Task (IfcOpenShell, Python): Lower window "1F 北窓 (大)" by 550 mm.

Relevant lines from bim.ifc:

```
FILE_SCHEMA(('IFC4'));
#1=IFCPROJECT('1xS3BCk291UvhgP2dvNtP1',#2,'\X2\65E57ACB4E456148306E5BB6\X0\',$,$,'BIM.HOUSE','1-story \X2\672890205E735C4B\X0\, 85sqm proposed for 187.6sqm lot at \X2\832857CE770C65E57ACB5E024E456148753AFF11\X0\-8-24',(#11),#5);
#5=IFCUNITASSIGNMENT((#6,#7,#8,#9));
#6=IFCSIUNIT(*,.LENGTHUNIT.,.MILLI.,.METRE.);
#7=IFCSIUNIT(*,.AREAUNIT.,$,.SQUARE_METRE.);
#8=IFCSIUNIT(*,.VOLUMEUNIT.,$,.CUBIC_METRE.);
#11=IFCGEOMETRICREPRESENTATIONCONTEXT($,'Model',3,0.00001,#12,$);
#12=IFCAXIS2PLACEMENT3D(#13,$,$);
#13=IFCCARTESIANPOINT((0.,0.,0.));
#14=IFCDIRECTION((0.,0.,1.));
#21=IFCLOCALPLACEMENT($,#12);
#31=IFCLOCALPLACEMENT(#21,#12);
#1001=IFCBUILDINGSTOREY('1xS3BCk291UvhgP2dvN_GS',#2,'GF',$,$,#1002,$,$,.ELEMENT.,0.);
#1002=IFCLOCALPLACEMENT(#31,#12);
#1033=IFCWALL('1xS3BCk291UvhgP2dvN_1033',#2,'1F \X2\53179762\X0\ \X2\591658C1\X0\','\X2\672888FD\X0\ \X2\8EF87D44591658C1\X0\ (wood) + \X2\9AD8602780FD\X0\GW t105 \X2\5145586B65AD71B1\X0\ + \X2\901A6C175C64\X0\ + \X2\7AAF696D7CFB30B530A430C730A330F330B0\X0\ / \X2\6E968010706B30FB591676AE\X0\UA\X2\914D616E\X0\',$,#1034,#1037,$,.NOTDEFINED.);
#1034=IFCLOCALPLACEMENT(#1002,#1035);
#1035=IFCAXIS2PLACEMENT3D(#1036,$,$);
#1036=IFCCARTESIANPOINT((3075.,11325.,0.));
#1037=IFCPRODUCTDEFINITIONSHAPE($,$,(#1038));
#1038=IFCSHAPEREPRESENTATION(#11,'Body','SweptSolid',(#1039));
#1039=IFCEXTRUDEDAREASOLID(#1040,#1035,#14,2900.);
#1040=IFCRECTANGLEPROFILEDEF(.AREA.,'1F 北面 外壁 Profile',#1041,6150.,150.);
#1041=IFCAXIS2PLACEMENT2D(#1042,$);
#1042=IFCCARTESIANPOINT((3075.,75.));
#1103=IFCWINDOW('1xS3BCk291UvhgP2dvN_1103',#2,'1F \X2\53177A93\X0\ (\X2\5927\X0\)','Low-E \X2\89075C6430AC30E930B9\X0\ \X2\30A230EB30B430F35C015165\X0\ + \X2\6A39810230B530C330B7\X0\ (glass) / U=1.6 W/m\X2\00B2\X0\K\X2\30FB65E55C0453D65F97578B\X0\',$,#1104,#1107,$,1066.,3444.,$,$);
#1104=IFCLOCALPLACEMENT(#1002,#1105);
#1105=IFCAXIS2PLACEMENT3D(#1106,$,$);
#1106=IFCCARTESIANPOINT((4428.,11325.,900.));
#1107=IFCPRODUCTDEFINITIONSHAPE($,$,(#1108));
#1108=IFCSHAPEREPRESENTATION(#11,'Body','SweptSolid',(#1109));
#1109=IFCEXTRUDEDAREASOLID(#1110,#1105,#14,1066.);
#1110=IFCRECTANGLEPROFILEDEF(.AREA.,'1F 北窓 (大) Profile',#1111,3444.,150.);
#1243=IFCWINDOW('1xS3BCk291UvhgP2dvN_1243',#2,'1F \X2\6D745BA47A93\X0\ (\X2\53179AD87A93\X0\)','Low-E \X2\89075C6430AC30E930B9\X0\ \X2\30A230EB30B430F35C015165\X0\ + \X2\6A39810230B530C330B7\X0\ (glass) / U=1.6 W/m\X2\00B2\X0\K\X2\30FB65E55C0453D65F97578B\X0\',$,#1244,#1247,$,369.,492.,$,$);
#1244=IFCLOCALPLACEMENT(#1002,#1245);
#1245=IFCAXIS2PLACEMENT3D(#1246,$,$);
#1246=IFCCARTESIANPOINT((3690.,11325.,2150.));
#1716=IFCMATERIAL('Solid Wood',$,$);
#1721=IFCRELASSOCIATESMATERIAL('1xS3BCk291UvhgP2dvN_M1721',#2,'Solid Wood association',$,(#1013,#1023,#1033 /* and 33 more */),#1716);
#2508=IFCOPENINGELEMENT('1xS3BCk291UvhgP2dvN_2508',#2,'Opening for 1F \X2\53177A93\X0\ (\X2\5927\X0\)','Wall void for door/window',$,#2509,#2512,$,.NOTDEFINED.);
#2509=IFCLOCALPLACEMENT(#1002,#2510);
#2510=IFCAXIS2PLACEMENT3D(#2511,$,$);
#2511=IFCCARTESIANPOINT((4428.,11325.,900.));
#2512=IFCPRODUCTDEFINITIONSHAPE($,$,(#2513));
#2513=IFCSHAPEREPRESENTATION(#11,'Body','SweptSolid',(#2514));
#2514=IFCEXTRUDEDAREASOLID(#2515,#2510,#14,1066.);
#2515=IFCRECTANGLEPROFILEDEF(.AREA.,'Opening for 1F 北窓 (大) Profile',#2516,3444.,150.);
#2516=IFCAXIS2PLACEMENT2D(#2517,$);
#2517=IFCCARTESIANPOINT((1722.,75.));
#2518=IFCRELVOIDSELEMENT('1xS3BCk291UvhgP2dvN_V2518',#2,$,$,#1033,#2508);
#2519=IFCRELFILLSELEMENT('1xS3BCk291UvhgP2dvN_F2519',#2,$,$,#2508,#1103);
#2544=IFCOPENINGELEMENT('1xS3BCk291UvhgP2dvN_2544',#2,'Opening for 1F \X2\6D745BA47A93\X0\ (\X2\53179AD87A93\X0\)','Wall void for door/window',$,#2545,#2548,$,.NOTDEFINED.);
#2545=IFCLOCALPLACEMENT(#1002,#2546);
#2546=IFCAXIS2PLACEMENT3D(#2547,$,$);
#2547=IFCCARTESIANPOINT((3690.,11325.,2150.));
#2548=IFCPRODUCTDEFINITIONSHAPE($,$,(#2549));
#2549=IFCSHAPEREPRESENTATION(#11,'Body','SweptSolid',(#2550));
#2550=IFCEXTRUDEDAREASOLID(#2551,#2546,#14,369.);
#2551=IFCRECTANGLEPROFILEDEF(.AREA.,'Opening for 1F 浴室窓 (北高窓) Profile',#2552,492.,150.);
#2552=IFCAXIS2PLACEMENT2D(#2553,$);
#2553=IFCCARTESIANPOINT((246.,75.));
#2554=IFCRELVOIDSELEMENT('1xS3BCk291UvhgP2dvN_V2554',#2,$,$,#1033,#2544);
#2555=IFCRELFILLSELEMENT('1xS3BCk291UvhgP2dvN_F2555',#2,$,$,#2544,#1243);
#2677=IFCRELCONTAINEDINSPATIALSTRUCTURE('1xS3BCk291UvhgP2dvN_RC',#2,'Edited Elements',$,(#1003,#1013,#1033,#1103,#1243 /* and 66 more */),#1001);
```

```python
import numpy as np
import ifcopenshell
import ifcopenshell.api.geometry
import ifcopenshell.util.placement
import ifcopenshell.util.unit

model = ifcopenshell.open("bim.ifc")
unit_scale = ifcopenshell.util.unit.calculate_unit_scale(model)

window = model.by_guid("1xS3BCk291UvhgP2dvN_1103")
opening = window.FillsVoids[0].RelatingOpeningElement
dz = -0.55 / unit_scale

shift = np.array([0.0, 0.0, dz])
# The window is not placed relative to its opening, so move both.
for product in (opening, window):
    matrix = ifcopenshell.util.placement.get_local_placement(product.ObjectPlacement)
    matrix[:3, 3] += shift
    ifcopenshell.api.geometry.edit_object_placement(model, product=product, matrix=matrix, is_si=False)

print(f"moved by {dz * unit_scale:+.3f} m")

model.write("bim-out.ifc")
```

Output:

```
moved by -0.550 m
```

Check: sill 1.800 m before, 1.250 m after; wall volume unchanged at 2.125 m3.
